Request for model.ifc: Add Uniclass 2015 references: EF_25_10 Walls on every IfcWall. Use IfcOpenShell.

First a look at what the model holds.

```python
import ifcopenshell

model = ifcopenshell.open("model.ifc")
print(model.schema)
print("classifications:", [c.Name for c in model.by_type("IfcClassification")])
for ifc_class in ("IfcDoor", "IfcRoof", "IfcStair", "IfcWall", "IfcWindow"):
    print(ifc_class, len(model.by_type(ifc_class)))
```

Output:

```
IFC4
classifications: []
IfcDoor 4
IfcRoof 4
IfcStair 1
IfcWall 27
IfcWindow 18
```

```python
import ifcopenshell
import ifcopenshell.api.classification

model = ifcopenshell.open("model.ifc")

system = ifcopenshell.api.classification.add_classification(model, classification="Uniclass 2015")

codes = {
    "IfcWall": ("EF_25_10", "Walls"),
}
for ifc_class, (code, name) in codes.items():
    products = model.by_type(ifc_class)
    ifcopenshell.api.classification.add_reference(
        model, products=products, classification=system, identification=code, name=name
    )
    print(code, len(products))

model.write("model_updated.ifc")
```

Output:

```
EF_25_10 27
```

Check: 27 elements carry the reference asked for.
